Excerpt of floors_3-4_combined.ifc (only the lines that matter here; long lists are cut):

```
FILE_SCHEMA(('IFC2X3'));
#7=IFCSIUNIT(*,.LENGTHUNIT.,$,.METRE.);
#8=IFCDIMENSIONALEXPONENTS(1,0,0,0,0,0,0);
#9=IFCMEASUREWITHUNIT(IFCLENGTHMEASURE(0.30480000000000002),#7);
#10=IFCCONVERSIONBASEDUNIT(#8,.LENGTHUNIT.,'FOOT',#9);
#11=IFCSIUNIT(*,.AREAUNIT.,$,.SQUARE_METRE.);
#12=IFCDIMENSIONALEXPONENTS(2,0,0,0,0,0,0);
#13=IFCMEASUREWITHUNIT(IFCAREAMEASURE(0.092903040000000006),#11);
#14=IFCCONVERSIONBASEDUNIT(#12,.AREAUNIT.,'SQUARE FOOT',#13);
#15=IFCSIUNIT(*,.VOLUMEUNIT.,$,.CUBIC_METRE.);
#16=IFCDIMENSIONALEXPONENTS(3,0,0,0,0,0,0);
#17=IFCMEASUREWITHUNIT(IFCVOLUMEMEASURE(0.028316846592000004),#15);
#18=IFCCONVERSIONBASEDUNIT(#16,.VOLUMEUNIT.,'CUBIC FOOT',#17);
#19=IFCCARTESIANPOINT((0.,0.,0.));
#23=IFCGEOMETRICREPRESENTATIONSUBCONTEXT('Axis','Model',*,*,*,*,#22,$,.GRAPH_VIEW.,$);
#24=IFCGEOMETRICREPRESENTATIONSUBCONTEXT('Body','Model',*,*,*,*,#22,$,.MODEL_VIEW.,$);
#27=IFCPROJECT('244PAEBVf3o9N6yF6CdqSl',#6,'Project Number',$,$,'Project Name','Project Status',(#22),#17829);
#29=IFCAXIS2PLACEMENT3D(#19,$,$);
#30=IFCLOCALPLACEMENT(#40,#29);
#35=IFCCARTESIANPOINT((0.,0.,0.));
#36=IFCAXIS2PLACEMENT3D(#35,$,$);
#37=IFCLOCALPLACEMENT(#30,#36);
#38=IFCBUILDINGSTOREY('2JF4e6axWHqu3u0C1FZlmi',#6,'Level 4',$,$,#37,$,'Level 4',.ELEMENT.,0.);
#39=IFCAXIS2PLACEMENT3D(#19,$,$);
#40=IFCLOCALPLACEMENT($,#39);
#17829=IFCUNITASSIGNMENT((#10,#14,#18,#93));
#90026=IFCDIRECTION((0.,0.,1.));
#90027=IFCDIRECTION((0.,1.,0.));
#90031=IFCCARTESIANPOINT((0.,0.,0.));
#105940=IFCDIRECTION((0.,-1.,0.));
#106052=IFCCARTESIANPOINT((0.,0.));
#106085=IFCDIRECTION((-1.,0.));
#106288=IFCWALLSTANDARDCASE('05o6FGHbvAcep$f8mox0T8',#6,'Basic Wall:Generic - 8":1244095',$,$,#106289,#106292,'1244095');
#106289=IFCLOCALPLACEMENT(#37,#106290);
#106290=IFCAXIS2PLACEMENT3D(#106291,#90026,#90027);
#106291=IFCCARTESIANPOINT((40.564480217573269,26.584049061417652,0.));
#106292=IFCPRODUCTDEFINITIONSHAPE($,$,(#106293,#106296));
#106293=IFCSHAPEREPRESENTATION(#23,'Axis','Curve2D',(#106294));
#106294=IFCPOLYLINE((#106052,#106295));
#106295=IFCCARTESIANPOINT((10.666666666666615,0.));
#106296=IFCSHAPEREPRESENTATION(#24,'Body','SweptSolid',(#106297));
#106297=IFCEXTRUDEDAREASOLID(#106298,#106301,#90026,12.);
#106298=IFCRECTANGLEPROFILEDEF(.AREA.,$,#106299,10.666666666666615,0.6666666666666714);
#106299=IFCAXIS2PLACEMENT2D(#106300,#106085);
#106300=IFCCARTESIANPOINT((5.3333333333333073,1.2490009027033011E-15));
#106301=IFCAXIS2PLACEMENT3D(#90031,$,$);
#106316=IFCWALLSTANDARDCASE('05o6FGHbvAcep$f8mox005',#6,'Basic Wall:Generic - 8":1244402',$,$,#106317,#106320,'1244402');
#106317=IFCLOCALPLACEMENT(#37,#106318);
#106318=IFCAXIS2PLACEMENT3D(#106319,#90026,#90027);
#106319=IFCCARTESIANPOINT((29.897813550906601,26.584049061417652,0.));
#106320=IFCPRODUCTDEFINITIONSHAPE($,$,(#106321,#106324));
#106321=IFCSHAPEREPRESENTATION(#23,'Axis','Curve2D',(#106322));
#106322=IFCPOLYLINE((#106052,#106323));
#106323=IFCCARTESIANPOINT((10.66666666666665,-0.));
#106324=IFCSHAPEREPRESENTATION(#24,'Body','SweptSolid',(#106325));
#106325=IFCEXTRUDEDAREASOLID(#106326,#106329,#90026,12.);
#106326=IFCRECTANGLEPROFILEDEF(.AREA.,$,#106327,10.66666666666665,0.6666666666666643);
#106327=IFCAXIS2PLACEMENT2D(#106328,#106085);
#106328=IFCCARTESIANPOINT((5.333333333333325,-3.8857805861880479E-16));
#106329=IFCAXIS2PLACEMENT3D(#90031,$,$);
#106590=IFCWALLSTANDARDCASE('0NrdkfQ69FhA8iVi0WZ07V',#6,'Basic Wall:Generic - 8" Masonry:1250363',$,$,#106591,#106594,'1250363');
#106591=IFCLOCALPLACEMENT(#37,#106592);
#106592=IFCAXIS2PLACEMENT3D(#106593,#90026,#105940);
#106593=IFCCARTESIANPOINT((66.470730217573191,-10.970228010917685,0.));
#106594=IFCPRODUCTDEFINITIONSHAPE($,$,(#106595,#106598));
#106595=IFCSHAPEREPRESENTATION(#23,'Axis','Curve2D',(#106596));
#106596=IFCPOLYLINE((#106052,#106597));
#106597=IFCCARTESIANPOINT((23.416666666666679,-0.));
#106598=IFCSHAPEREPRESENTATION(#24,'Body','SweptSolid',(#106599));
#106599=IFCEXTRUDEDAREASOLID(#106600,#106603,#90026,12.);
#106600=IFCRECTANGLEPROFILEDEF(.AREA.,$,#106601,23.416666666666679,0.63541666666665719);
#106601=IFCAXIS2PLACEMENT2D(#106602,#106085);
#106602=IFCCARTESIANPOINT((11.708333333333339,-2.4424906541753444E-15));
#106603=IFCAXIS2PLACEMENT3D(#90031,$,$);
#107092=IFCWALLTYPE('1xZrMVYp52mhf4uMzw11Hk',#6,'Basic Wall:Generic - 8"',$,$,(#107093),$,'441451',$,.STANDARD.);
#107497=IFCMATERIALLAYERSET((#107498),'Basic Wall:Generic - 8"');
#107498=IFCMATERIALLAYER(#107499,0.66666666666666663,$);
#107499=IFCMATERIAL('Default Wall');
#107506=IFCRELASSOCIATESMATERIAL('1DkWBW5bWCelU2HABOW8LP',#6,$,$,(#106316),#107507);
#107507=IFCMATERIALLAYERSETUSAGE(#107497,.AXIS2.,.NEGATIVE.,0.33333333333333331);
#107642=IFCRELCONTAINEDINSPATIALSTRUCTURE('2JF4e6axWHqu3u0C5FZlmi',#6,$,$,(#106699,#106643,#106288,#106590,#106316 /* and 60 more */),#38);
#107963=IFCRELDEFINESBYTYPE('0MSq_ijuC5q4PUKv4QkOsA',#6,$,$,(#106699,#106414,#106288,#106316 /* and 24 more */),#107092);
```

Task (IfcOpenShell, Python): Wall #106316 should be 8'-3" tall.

```python
import ifcopenshell
import ifcopenshell.geom
import ifcopenshell.util.representation
import ifcopenshell.util.shape
import ifcopenshell.util.unit

model = ifcopenshell.open("floors_3-4_combined.ifc")
unit_scale = ifcopenshell.util.unit.calculate_unit_scale(model)
settings = ifcopenshell.geom.settings()


def volume(element):
    """Net volume in cubic metres, openings subtracted."""
    shape = ifcopenshell.geom.create_shape(settings, element)
    return ifcopenshell.util.shape.get_volume(shape.geometry)


wall = model.by_id(106316)
before = volume(wall)

body = ifcopenshell.util.representation.get_representation(wall, "Model", "Body")
solid = body.Items[0]
old_height = solid.Depth
solid.Depth = 99 * 0.0254 / unit_scale
after = volume(wall)

print(f"height {old_height:g} -> {solid.Depth:g}, volume {before:.3f} -> {after:.3f} m3")

model.write("floors_3-4_combined-out.ifc")
```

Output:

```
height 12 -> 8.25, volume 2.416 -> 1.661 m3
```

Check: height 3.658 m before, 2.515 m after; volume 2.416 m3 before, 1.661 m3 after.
